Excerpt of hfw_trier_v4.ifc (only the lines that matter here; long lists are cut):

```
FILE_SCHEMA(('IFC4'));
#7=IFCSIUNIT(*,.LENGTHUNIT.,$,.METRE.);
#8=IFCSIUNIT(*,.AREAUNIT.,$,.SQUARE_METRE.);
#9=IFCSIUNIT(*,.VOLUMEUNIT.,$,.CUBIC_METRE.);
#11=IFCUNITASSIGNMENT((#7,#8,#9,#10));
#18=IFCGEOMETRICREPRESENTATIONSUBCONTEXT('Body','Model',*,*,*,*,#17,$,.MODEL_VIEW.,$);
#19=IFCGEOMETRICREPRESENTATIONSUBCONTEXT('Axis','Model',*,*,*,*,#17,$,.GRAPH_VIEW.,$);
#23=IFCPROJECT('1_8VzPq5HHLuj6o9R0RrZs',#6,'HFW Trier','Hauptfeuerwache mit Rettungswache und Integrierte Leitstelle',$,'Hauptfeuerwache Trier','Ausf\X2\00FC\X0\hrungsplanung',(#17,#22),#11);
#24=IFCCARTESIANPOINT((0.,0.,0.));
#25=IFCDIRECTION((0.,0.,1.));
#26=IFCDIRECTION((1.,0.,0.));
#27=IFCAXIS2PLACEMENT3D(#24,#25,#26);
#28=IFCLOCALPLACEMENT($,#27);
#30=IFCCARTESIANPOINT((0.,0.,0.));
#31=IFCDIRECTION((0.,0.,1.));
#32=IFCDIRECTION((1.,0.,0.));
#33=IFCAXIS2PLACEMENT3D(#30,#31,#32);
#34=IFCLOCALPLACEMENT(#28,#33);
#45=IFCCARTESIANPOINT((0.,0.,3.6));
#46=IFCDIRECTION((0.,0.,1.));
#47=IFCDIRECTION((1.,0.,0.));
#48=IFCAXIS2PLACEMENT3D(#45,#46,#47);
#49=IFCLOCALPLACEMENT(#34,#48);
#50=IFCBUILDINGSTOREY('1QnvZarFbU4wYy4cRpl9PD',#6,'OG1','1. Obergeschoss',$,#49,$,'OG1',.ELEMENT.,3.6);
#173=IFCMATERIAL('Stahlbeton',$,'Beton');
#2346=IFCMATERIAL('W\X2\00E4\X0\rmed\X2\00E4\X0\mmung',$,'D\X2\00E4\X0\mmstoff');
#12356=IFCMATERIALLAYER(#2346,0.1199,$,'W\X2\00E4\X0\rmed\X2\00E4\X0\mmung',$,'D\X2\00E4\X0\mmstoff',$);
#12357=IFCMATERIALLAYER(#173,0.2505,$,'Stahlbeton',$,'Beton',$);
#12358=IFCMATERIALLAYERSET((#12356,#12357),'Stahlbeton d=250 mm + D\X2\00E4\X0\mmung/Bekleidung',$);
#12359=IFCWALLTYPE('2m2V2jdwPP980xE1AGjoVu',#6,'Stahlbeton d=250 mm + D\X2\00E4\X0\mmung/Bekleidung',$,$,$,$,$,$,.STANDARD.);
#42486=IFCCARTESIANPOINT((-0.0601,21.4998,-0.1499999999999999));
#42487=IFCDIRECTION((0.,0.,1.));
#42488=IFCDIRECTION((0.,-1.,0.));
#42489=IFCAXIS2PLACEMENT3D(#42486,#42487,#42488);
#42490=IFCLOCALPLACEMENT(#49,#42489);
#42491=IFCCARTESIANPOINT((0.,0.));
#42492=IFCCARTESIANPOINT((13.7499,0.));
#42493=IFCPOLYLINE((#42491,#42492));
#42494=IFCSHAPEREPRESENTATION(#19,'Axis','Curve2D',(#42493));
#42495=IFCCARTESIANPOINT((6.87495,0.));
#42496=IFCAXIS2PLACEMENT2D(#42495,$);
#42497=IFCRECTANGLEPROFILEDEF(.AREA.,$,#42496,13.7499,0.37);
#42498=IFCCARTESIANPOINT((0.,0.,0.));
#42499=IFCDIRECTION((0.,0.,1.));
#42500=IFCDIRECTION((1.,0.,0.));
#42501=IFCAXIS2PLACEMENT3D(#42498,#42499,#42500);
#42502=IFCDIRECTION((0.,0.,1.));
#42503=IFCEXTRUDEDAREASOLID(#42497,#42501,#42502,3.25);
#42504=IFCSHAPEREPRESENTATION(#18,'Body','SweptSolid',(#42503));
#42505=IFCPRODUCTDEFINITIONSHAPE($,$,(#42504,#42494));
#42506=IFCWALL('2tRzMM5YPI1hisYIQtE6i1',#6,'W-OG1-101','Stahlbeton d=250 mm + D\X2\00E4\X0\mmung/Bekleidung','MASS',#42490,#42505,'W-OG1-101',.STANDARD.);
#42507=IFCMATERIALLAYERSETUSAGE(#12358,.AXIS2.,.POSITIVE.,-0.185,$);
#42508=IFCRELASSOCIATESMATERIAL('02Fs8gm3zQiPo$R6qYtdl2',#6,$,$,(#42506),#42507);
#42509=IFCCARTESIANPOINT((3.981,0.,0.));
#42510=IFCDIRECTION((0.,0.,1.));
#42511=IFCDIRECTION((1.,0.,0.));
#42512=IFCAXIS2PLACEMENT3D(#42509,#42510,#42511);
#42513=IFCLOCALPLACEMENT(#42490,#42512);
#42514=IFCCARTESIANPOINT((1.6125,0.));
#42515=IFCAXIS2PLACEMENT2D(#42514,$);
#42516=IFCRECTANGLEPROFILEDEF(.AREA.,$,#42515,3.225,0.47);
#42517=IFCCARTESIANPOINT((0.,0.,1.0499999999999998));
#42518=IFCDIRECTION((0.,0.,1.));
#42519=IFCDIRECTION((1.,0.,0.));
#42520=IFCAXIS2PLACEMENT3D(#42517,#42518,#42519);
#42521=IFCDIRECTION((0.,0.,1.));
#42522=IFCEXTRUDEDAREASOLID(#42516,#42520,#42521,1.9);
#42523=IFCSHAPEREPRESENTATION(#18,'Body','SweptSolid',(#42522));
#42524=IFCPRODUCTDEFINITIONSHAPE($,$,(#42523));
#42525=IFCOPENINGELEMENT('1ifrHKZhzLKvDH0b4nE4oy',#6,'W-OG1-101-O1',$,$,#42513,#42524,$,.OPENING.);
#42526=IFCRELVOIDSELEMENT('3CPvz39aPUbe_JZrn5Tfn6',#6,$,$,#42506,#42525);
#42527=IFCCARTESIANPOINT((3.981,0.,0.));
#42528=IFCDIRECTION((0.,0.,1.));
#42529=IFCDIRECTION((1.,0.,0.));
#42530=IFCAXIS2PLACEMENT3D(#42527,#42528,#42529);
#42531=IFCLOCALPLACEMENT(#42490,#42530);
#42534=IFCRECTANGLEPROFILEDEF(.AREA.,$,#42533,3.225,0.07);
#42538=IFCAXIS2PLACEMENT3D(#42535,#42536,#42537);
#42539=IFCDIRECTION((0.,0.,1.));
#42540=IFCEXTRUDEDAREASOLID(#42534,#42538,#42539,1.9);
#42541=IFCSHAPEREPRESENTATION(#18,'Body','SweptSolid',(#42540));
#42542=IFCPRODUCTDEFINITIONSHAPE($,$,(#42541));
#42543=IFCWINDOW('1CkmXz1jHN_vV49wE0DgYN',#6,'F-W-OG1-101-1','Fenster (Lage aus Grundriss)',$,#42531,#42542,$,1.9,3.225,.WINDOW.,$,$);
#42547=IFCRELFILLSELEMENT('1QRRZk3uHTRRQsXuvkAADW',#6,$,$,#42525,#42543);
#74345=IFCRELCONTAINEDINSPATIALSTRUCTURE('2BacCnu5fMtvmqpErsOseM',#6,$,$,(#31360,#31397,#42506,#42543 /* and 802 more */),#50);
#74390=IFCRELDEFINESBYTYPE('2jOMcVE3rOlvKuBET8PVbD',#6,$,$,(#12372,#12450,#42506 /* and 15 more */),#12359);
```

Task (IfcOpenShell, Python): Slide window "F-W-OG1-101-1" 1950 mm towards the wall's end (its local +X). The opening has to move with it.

```python
import ifcopenshell
import ifcopenshell.api.geometry
import ifcopenshell.util.placement

model = ifcopenshell.open("hfw_trier_v4.ifc")

window = model.by_guid("1CkmXz1jHN_vV49wE0DgYN")
opening = window.FillsVoids[0].RelatingOpeningElement
wall = opening.VoidsElements[0].RelatingBuildingElement

wall_matrix = ifcopenshell.util.placement.get_local_placement(wall.ObjectPlacement)
shift = wall_matrix[:3, 0] * 1.95
before = ifcopenshell.util.placement.get_local_placement(window.ObjectPlacement)[:3, 3].copy()

# The window is not placed relative to its opening, so move both.
for product in (opening, window):
    matrix = ifcopenshell.util.placement.get_local_placement(product.ObjectPlacement)
    matrix[:3, 3] += shift
    ifcopenshell.api.geometry.edit_object_placement(model, product=product, matrix=matrix, is_si=False)

after = ifcopenshell.util.placement.get_local_placement(window.ObjectPlacement)[:3, 3]
print("window moved by", (after - before).round(3) + 0.0)

model.write("hfw_trier_v4-out.ifc")
```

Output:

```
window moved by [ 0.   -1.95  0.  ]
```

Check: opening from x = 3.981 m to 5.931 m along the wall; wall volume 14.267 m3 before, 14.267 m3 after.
